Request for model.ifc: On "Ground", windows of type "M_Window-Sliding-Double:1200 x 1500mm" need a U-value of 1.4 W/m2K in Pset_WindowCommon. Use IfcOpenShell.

First a look at what the model holds.

```python
import ifcopenshell
import ifcopenshell.util.element

model = ifcopenshell.open("model.ifc")
print(model.schema)
storey = next(s for s in model.by_type("IfcBuildingStorey") if s.Name == "Ground")
windows = [e for e in ifcopenshell.util.element.get_decomposition(storey) if e.is_a("IfcWindow")]
seen = {}
for e in windows:
    element_type = ifcopenshell.util.element.get_type(e)
    key = (element_type.Name if element_type != e and element_type else None, ifcopenshell.util.element.get_pset(e, "Pset_WindowCommon", "ThermalTransmittance"))
    seen[key] = seen.get(key, 0) + 1
for (name, value), count in sorted(seen.items(), key=str):
    print(count, "x", name, "|", value)
```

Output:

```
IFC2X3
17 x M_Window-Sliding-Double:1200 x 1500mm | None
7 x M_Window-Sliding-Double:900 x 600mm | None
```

```python
import ifcopenshell
import ifcopenshell.api.pset
import ifcopenshell.util.element

model = ifcopenshell.open("model.ifc")

storey = next(s for s in model.by_type("IfcBuildingStorey") if s.Name == "Ground")
windows = [e for e in ifcopenshell.util.element.get_decomposition(storey) if e.is_a("IfcWindow")]

count = 0
for e in windows:
    element_type = ifcopenshell.util.element.get_type(e)
    if element_type in (None, e) or element_type.Name != "M_Window-Sliding-Double:1200 x 1500mm":
        continue
    # add_pset returns the element's existing set when there is one.
    pset = ifcopenshell.api.pset.add_pset(model, product=e, name="Pset_WindowCommon")
    ifcopenshell.api.pset.edit_pset(model, pset=pset, properties={"ThermalTransmittance": 1.4})
    count += 1

print(count, "windows updated")

model.write("model_v2.ifc")
```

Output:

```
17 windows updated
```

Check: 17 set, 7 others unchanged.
